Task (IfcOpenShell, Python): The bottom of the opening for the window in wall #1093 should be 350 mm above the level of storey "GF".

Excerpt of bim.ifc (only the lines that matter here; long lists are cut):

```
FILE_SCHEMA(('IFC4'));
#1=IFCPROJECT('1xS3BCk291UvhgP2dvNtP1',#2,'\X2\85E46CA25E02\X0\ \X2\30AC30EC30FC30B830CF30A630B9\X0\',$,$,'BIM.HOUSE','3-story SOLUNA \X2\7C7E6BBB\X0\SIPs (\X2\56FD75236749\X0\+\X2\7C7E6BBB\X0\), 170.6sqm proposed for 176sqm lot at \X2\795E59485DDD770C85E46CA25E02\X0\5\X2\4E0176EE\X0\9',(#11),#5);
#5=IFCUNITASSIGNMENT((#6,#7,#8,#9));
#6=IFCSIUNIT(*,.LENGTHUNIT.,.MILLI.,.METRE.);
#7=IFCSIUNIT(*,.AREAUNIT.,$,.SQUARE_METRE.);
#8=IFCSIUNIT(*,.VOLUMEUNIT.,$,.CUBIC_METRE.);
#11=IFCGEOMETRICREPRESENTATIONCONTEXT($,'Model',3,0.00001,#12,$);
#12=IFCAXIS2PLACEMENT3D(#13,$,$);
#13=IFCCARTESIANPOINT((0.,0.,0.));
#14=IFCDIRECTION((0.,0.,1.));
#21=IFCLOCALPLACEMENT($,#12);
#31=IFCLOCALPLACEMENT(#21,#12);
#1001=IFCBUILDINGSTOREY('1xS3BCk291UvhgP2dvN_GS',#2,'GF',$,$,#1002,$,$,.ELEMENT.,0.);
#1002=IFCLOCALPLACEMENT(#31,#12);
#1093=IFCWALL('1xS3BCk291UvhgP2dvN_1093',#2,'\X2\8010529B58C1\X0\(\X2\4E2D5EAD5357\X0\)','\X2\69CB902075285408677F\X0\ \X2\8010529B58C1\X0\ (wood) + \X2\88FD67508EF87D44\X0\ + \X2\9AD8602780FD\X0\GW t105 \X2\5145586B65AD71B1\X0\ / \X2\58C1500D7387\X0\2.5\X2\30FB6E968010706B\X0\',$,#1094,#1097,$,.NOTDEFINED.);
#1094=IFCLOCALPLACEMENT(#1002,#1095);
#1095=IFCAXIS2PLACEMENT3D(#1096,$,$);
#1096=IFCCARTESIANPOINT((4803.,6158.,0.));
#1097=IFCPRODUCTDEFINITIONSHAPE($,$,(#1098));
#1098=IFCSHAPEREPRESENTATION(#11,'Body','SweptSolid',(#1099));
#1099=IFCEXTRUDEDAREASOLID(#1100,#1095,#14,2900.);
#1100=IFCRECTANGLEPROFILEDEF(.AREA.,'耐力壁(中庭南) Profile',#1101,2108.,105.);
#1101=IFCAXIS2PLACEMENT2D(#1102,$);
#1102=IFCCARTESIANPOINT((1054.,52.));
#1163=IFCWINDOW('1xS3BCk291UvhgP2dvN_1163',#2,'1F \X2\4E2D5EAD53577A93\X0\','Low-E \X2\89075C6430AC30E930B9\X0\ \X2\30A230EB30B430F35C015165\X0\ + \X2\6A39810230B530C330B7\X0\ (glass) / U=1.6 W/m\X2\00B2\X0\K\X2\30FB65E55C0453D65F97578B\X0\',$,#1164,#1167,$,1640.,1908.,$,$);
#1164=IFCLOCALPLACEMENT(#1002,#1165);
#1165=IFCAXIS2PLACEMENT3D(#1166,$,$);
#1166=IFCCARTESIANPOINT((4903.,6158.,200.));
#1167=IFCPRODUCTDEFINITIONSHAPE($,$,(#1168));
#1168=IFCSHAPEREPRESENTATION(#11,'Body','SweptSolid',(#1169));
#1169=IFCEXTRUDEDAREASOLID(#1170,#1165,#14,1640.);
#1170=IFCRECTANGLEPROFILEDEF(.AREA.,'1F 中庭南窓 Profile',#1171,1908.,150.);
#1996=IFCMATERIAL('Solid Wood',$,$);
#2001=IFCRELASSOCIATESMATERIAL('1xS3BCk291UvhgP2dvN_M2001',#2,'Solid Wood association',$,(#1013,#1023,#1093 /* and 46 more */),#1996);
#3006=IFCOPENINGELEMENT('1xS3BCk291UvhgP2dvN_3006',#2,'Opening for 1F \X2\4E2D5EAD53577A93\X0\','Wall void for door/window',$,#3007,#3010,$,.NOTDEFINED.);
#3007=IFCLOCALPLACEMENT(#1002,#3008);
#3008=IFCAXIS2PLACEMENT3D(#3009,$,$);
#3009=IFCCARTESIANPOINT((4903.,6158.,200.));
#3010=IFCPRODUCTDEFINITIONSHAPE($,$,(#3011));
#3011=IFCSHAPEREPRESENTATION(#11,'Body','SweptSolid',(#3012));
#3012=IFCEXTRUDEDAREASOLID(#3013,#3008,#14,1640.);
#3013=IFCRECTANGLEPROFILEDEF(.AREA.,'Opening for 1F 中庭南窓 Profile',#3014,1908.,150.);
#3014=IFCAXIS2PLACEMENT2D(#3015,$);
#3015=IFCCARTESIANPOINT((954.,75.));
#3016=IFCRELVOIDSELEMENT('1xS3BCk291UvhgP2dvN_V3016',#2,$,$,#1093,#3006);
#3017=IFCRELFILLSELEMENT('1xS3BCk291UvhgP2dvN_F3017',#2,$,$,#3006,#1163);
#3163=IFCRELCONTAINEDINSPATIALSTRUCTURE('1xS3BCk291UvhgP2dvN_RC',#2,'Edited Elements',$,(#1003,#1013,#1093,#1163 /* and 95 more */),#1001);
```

```python
import numpy as np
import ifcopenshell
import ifcopenshell.api.geometry
import ifcopenshell.geom
import ifcopenshell.util.element
import ifcopenshell.util.placement
import ifcopenshell.util.shape
import ifcopenshell.util.unit

model = ifcopenshell.open("bim.ifc")
unit_scale = ifcopenshell.util.unit.calculate_unit_scale(model)

window = model.by_id(1163)
opening = window.FillsVoids[0].RelatingOpeningElement
storey = ifcopenshell.util.element.get_container(window, ifc_class="IfcBuildingStorey")
level = ifcopenshell.util.placement.get_local_placement(storey.ObjectPlacement)[2, 3]

# The opening's origin need not be at the sill, so measure its lowest point.
shape = ifcopenshell.geom.create_shape(ifcopenshell.geom.settings(), opening)
bottom = ifcopenshell.util.shape.get_shape_bottom_elevation(shape, shape.geometry) / unit_scale
dz = level + 0.35 / unit_scale - bottom

shift = np.array([0.0, 0.0, dz])
# The window is not placed relative to its opening, so move both.
for product in (opening, window):
    matrix = ifcopenshell.util.placement.get_local_placement(product.ObjectPlacement)
    matrix[:3, 3] += shift
    ifcopenshell.api.geometry.edit_object_placement(model, product=product, matrix=matrix, is_si=False)

print(f"moved by {dz * unit_scale:+.3f} m")

model.write("bim_edited.ifc")
```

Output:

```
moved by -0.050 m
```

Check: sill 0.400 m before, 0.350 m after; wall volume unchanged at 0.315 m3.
